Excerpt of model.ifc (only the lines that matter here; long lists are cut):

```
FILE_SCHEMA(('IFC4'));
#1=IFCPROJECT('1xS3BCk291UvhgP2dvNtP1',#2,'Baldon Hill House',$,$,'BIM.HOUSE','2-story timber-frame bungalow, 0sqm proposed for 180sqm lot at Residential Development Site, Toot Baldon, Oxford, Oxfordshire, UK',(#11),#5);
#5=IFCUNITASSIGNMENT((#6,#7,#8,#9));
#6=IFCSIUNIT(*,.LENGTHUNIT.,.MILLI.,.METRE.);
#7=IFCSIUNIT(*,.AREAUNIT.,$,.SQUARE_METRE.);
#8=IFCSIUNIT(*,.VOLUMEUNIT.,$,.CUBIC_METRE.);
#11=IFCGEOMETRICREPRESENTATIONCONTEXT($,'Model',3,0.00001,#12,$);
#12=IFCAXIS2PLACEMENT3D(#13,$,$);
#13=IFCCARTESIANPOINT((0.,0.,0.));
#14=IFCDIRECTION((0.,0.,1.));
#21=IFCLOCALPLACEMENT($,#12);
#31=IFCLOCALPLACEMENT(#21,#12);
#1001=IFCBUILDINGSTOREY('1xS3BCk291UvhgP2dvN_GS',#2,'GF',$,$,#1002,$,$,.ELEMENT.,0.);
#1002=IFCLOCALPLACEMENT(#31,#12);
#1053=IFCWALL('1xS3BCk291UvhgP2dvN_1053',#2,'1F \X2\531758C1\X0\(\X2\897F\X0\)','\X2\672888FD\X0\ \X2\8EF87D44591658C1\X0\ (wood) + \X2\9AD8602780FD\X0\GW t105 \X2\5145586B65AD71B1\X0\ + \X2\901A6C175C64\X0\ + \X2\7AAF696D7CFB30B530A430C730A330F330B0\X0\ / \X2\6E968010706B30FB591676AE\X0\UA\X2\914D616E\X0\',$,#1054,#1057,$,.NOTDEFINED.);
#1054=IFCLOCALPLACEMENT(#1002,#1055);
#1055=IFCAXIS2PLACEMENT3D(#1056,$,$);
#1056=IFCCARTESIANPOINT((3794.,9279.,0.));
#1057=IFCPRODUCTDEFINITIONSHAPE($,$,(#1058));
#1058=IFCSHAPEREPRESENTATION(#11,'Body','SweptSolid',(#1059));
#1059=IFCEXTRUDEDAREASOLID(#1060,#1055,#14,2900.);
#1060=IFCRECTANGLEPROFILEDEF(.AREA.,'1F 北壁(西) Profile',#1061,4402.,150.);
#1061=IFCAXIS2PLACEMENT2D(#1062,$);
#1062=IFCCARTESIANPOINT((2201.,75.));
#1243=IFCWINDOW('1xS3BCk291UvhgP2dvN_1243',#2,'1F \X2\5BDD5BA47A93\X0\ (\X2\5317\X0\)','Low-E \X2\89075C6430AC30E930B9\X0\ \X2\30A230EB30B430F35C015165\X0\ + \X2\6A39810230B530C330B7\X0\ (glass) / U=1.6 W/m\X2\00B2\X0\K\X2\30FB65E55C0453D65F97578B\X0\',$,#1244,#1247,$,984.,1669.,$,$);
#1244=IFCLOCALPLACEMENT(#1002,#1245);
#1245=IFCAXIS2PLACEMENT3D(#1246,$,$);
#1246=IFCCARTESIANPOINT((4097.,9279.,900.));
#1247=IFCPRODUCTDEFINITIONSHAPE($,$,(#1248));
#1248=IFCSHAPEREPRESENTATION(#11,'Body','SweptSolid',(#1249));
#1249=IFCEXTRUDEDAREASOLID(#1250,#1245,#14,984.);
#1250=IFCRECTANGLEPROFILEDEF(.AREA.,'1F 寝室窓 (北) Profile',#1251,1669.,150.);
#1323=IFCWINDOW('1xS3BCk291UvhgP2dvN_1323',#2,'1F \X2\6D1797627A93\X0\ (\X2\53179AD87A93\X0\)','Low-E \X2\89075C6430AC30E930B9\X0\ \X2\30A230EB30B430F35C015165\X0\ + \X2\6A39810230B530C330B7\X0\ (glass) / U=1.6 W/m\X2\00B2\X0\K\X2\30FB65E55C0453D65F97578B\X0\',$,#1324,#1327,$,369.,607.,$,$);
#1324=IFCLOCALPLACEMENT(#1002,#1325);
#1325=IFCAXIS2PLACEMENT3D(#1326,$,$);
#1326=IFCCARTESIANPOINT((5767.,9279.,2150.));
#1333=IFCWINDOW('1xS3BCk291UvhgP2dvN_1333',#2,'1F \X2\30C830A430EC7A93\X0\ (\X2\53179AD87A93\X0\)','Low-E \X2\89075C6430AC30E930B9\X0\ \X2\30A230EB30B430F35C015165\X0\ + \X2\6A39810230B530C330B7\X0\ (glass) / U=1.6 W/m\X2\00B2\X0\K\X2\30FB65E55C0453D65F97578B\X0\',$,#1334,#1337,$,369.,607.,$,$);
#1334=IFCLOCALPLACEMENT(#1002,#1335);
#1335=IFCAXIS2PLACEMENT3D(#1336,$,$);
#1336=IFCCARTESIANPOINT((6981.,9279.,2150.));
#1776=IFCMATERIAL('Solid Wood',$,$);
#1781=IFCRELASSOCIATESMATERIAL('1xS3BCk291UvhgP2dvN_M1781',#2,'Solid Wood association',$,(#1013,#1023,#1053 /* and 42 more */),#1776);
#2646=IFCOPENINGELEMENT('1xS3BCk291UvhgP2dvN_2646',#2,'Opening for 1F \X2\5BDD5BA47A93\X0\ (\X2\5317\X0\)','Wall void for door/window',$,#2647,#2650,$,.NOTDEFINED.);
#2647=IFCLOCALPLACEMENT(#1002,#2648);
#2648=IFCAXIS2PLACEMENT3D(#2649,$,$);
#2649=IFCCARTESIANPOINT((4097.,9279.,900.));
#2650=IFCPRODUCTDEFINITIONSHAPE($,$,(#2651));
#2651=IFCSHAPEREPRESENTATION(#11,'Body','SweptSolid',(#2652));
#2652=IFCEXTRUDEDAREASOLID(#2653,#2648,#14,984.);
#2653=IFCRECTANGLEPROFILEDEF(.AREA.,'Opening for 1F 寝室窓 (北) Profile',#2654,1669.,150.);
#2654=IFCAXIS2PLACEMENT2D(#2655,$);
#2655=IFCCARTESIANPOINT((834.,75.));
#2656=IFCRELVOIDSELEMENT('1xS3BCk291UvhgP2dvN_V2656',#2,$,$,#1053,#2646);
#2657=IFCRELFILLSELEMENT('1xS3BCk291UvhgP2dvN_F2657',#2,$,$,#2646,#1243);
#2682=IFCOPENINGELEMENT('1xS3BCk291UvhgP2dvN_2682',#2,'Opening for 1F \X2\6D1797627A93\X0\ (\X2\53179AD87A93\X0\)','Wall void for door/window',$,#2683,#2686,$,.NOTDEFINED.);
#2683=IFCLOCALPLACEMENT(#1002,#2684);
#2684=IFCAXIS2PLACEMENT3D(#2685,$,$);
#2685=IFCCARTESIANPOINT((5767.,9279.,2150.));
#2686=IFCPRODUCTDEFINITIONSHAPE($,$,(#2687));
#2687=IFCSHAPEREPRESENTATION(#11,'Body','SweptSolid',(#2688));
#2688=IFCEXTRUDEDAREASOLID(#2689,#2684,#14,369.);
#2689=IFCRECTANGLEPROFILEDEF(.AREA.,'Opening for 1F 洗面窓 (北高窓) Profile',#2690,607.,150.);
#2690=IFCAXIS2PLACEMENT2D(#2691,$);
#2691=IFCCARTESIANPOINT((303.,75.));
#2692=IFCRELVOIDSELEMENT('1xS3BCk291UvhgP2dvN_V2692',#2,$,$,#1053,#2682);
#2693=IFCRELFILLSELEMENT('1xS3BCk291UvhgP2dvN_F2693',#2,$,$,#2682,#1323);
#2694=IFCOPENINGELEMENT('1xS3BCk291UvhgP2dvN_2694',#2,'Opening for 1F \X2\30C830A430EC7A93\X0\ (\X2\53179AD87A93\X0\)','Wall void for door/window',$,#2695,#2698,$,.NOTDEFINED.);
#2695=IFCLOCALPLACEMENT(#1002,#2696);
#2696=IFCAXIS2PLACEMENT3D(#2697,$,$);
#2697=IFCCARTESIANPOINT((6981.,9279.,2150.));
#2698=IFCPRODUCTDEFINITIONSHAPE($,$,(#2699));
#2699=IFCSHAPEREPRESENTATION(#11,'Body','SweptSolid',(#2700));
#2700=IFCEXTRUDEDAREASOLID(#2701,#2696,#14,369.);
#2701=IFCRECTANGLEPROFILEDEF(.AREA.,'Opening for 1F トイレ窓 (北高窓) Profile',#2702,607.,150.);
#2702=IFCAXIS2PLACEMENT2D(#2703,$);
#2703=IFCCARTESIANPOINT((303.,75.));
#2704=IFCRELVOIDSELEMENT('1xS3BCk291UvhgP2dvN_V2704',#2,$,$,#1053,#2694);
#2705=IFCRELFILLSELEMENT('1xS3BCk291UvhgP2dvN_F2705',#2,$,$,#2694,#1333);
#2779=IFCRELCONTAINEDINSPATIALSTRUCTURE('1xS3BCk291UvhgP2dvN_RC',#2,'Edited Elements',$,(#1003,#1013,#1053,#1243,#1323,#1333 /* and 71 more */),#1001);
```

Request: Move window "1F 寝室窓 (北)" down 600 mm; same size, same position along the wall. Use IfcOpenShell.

```python
import numpy as np
import ifcopenshell
import ifcopenshell.api.geometry
import ifcopenshell.util.placement
import ifcopenshell.util.unit

model = ifcopenshell.open("model.ifc")
unit_scale = ifcopenshell.util.unit.calculate_unit_scale(model)

window = model.by_guid("1xS3BCk291UvhgP2dvN_1243")
opening = window.FillsVoids[0].RelatingOpeningElement
dz = -0.6 / unit_scale

shift = np.array([0.0, 0.0, dz])
# The window is not placed relative to its opening, so move both.
for product in (opening, window):
    matrix = ifcopenshell.util.placement.get_local_placement(product.ObjectPlacement)
    matrix[:3, 3] += shift
    ifcopenshell.api.geometry.edit_object_placement(model, product=product, matrix=matrix, is_si=False)

print(f"moved by {dz * unit_scale:+.3f} m")

model.write("model-out.ifc")
```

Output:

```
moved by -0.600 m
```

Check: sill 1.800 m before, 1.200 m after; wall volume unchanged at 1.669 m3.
